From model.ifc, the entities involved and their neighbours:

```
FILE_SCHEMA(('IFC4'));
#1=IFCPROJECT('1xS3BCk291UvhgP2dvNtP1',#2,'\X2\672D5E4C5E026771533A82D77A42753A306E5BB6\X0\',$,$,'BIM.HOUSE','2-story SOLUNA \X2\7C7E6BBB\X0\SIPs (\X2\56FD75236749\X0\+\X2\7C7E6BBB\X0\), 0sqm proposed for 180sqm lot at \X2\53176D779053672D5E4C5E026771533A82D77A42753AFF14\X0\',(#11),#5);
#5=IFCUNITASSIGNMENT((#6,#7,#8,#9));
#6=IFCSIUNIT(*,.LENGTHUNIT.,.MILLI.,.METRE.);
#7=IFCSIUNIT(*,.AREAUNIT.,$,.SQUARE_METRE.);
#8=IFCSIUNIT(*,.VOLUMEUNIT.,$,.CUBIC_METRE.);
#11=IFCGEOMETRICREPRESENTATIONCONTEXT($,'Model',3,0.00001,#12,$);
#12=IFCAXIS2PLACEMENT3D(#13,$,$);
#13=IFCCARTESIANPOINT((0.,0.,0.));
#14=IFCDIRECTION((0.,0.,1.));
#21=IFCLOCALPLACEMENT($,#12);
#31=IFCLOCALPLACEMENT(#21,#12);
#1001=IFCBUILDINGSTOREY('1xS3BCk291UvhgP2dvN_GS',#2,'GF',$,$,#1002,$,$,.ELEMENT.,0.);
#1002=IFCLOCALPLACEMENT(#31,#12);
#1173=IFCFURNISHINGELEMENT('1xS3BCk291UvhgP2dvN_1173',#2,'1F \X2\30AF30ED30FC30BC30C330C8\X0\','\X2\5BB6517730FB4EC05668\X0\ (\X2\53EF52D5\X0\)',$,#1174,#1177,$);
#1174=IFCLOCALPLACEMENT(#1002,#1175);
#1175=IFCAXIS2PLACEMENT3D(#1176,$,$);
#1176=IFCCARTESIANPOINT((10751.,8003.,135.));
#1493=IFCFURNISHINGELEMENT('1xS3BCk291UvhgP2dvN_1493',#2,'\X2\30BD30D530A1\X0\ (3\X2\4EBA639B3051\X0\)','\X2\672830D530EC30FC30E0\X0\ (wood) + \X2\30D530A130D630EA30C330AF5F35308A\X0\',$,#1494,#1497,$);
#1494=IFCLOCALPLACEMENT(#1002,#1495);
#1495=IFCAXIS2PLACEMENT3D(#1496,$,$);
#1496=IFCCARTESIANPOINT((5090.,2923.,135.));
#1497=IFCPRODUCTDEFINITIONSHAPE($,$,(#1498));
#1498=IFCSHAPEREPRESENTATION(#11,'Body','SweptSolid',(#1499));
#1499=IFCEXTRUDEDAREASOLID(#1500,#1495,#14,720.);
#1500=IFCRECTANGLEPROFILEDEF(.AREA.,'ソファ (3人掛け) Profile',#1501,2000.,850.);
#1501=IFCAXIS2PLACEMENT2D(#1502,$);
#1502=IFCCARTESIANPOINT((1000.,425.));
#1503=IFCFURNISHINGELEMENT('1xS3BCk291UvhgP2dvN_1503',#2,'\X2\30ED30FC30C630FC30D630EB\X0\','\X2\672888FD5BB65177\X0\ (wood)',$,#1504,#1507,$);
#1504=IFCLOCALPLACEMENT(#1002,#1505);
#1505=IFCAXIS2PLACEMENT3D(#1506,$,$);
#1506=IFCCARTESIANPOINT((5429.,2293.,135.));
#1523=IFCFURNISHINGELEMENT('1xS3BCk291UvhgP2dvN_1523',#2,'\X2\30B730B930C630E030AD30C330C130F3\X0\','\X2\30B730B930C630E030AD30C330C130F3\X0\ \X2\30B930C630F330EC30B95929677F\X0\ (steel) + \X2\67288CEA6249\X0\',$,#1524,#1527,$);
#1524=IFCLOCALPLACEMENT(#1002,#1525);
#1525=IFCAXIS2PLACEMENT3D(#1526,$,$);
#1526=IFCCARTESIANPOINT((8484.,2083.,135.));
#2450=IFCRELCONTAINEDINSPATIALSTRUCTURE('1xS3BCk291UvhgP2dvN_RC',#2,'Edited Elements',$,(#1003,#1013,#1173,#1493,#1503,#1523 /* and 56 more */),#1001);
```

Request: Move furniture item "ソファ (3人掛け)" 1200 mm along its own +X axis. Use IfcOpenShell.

```python
import ifcopenshell
import ifcopenshell.api.geometry
import ifcopenshell.util.placement
import ifcopenshell.util.unit

model = ifcopenshell.open("model.ifc")
unit_scale = ifcopenshell.util.unit.calculate_unit_scale(model)

item = model.by_guid("1xS3BCk291UvhgP2dvN_1493")
matrix = ifcopenshell.util.placement.get_local_placement(item.ObjectPlacement)
matrix[:3, 3] += matrix[:3, 0] * 1.2 / unit_scale
ifcopenshell.api.geometry.edit_object_placement(model, product=item, matrix=matrix, is_si=False)

print(ifcopenshell.util.placement.get_local_placement(item.ObjectPlacement).round(3) + 0.0)

model.write("model_v2.ifc")
```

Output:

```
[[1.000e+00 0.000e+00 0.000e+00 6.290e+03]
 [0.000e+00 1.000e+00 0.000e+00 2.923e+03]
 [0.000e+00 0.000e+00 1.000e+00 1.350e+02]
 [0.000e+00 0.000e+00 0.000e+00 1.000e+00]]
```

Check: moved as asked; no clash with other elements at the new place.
